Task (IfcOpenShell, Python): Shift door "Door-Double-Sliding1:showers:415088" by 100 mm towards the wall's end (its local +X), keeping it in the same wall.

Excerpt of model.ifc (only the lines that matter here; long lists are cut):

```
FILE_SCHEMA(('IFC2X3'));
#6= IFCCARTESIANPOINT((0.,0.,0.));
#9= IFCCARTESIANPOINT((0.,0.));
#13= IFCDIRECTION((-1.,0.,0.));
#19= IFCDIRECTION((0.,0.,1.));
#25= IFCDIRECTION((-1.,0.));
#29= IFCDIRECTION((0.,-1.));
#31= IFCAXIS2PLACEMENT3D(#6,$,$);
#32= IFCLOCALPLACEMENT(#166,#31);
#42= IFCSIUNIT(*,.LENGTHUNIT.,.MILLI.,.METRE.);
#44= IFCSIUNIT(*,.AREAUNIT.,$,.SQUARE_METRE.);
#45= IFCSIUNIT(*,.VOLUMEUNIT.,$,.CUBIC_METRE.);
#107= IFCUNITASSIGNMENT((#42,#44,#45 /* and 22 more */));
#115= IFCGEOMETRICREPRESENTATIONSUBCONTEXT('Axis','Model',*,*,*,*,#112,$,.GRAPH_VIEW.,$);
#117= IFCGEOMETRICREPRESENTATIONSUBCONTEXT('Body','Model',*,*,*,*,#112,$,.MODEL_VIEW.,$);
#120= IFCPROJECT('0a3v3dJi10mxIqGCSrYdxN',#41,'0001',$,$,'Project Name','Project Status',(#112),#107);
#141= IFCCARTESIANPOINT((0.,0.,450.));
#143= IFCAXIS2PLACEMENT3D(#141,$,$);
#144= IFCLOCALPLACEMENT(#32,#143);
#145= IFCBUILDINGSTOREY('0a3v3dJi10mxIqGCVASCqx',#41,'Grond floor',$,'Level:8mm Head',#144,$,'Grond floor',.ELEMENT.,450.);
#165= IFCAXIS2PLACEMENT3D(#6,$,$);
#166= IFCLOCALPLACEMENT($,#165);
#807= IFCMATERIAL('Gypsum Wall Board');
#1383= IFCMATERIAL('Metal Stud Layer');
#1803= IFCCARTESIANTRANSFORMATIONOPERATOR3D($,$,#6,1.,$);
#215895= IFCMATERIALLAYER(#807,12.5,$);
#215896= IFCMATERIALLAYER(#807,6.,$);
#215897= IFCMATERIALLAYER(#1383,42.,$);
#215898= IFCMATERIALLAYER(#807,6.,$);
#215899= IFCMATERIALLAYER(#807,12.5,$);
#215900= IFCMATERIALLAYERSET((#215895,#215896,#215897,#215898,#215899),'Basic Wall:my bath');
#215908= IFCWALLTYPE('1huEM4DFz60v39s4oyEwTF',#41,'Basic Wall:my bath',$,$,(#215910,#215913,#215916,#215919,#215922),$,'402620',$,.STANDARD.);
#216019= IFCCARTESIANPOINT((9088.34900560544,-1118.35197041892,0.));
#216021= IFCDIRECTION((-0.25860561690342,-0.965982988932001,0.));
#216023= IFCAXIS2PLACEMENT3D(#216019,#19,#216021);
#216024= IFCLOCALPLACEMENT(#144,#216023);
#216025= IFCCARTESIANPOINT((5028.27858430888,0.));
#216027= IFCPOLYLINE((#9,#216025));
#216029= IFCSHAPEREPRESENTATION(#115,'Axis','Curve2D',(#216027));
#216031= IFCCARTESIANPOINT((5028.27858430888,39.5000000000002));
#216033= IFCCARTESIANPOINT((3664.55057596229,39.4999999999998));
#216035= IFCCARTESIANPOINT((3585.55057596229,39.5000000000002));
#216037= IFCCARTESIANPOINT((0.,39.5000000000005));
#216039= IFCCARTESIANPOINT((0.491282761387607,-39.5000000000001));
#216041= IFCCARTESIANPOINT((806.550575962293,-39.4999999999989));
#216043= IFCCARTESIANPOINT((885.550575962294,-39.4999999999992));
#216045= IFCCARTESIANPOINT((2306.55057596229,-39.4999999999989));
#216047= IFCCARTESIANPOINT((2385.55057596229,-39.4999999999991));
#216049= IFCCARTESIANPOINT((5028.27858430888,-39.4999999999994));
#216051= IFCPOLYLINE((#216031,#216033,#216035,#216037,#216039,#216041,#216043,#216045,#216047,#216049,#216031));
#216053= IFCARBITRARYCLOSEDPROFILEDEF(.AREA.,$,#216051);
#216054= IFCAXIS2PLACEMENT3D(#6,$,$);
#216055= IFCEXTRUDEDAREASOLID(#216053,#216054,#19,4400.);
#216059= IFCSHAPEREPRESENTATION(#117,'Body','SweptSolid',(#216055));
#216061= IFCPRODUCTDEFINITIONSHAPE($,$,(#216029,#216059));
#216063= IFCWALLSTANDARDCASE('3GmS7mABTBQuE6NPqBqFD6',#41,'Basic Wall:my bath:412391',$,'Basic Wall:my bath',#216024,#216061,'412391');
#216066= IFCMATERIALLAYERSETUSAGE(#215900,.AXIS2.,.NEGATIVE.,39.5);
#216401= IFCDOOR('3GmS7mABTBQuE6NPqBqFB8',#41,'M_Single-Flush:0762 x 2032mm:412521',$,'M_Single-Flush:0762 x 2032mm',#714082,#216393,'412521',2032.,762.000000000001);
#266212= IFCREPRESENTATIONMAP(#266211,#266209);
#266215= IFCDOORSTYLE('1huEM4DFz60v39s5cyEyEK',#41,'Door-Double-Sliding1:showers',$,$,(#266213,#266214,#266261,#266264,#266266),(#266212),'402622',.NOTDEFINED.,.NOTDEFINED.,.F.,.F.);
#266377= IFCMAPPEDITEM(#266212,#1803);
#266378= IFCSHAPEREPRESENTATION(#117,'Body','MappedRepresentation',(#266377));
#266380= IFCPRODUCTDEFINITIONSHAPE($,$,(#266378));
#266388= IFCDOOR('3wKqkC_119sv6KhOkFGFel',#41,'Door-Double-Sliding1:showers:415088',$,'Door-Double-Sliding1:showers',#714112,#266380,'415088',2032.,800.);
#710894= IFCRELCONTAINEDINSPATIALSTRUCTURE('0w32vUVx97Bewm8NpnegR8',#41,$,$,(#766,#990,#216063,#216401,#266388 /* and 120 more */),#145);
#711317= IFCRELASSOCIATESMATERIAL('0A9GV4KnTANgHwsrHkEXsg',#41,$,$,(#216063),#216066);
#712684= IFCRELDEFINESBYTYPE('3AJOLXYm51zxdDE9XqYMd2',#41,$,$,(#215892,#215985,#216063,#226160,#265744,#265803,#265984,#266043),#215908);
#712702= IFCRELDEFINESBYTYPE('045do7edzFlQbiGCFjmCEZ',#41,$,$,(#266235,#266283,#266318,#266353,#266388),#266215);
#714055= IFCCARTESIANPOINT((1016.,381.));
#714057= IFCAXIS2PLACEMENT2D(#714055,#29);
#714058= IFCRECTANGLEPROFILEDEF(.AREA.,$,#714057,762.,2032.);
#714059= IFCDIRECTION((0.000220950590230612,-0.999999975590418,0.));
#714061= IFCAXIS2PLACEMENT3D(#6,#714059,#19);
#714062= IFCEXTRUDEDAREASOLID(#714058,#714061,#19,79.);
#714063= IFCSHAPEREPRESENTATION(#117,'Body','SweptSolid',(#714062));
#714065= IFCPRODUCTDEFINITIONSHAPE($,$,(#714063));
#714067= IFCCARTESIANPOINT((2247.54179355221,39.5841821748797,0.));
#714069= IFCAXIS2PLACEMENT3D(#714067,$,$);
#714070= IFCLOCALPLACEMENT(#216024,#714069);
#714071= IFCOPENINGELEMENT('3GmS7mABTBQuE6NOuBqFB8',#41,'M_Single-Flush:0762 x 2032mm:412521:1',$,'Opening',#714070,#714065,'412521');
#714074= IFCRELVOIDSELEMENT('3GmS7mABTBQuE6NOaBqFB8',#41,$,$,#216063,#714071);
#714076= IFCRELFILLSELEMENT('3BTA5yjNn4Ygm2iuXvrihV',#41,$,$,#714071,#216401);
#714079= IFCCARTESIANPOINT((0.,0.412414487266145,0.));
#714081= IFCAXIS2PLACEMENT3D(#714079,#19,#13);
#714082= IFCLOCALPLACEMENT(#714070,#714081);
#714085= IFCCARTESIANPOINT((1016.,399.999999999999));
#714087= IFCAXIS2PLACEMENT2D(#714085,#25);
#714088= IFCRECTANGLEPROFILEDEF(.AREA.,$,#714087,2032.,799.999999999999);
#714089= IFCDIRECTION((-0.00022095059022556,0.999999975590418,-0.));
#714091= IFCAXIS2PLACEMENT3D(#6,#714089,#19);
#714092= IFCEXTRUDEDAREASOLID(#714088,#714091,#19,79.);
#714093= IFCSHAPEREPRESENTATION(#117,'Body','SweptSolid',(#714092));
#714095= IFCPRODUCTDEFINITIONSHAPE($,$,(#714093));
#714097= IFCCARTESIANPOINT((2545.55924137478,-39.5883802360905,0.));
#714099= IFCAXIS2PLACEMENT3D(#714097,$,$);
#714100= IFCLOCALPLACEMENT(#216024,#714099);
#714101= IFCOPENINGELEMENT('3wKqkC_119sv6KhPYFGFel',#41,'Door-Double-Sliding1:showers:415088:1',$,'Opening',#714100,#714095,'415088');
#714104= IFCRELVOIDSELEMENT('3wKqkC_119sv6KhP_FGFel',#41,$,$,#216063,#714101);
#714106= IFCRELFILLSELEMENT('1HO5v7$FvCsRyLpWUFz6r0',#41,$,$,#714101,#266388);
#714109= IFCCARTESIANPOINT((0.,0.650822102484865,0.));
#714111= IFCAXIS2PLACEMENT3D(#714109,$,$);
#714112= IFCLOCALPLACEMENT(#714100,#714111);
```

```python
import ifcopenshell
import ifcopenshell.api.geometry
import ifcopenshell.util.placement
import ifcopenshell.util.unit

model = ifcopenshell.open("model.ifc")
unit_scale = ifcopenshell.util.unit.calculate_unit_scale(model)

door = model.by_id(266388)
opening = door.FillsVoids[0].RelatingOpeningElement
wall = opening.VoidsElements[0].RelatingBuildingElement

wall_matrix = ifcopenshell.util.placement.get_local_placement(wall.ObjectPlacement)
shift = wall_matrix[:3, 0] * 0.1 / unit_scale
before = ifcopenshell.util.placement.get_local_placement(door.ObjectPlacement)[:3, 3].copy()

# The door is placed relative to its opening, so it follows when the opening moves.
matrix = ifcopenshell.util.placement.get_local_placement(opening.ObjectPlacement)
matrix[:3, 3] += shift
ifcopenshell.api.geometry.edit_object_placement(
    model, product=opening, matrix=matrix, is_si=False, should_transform_children=True
)

after = ifcopenshell.util.placement.get_local_placement(door.ObjectPlacement)[:3, 3]
print("door moved by", (after - before).round(3) + 0.0)

model.write("model-out.ifc")
```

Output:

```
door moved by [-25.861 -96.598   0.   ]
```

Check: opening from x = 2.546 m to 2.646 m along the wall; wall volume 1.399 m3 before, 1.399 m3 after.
